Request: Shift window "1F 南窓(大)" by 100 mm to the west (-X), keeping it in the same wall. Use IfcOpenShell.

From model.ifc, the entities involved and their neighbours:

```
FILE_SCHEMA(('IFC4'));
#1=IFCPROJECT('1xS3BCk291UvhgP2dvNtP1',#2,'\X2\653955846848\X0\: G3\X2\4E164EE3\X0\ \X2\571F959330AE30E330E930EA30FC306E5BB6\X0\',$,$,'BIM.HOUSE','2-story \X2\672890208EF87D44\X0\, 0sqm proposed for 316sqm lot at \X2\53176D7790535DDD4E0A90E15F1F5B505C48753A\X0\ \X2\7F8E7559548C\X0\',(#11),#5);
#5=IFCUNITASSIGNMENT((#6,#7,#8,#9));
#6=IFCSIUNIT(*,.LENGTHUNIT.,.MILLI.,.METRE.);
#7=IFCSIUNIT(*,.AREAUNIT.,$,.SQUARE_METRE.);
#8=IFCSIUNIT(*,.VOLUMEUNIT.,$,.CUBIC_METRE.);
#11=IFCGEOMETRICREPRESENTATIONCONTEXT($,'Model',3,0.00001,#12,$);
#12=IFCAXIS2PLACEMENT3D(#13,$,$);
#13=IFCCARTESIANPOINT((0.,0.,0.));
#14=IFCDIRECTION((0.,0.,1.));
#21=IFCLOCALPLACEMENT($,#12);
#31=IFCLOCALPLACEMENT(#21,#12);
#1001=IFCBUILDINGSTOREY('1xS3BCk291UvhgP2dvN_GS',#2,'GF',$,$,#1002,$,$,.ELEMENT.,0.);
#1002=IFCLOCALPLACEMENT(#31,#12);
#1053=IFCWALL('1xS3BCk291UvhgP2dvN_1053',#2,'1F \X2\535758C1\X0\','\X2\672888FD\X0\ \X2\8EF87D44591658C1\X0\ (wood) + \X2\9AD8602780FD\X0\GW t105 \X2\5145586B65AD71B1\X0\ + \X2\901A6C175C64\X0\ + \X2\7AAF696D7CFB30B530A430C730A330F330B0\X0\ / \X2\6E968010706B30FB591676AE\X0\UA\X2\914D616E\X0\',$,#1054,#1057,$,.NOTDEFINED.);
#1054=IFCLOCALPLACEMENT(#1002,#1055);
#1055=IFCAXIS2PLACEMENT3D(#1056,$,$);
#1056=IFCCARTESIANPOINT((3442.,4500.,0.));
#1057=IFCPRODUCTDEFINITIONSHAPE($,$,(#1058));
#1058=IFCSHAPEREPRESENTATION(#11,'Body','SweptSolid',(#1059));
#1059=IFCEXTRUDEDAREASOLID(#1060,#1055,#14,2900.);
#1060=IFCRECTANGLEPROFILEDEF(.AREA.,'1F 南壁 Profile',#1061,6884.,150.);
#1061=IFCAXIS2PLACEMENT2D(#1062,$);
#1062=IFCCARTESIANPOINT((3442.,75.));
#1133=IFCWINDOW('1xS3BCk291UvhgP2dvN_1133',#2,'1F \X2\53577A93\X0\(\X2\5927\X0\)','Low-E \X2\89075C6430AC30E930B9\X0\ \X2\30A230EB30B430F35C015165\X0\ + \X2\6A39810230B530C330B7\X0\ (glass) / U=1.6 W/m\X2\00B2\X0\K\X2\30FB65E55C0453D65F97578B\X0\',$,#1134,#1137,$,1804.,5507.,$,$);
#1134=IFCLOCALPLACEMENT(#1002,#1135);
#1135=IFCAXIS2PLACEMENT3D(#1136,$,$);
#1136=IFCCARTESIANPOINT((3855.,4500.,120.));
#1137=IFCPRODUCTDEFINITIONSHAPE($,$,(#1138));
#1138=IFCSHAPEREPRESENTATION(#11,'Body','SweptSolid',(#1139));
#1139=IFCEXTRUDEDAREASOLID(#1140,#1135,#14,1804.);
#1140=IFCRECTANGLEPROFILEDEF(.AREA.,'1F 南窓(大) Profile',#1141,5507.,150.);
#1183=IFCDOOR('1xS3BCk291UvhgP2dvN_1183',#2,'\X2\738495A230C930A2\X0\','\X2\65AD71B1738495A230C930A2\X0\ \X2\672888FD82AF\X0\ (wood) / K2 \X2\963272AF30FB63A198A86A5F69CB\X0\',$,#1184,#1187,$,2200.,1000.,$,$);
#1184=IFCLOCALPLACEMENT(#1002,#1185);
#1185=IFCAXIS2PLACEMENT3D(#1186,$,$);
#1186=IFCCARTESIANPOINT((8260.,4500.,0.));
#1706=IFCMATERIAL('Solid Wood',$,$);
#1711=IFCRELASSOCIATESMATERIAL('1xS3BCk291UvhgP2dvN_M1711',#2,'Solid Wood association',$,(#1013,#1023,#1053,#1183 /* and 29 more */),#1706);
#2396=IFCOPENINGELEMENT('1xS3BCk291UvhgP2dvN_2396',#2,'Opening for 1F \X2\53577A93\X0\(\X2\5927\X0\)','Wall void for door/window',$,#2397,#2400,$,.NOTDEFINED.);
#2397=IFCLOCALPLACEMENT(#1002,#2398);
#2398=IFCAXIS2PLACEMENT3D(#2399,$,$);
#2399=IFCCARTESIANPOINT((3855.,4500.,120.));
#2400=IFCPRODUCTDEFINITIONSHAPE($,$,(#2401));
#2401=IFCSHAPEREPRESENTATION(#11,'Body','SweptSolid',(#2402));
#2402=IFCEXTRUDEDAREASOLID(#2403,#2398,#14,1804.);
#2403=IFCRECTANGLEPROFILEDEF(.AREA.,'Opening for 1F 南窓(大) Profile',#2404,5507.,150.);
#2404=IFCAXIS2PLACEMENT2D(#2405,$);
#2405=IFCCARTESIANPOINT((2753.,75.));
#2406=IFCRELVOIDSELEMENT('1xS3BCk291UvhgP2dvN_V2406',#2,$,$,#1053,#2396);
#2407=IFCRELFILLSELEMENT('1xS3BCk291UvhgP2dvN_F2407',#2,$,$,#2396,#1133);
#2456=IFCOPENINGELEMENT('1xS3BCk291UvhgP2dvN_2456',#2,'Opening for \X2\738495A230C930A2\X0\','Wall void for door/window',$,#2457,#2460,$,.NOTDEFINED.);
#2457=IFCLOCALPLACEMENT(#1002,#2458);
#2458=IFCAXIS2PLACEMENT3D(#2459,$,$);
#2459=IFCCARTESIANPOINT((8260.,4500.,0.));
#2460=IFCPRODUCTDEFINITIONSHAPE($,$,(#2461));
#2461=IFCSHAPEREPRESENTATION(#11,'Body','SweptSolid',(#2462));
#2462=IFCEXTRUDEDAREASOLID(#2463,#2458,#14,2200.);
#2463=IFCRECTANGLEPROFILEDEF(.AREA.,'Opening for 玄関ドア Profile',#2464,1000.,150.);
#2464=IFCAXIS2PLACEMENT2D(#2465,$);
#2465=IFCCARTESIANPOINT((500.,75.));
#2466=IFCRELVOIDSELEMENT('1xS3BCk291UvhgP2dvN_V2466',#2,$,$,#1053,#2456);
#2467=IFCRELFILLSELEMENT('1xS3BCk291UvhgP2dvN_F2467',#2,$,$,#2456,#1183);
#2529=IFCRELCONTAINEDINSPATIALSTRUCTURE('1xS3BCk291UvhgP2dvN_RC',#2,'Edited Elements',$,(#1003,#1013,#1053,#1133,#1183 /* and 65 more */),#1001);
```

```python
import ifcopenshell
import ifcopenshell.api.geometry
import ifcopenshell.util.placement
import ifcopenshell.util.unit

model = ifcopenshell.open("model.ifc")
unit_scale = ifcopenshell.util.unit.calculate_unit_scale(model)

window = model.by_guid("1xS3BCk291UvhgP2dvN_1133")
opening = window.FillsVoids[0].RelatingOpeningElement
wall = opening.VoidsElements[0].RelatingBuildingElement

wall_matrix = ifcopenshell.util.placement.get_local_placement(wall.ObjectPlacement)
shift = wall_matrix[:3, 0] * -0.1 / unit_scale
before = ifcopenshell.util.placement.get_local_placement(window.ObjectPlacement)[:3, 3].copy()

# The window is not placed relative to its opening, so move both.
for product in (opening, window):
    matrix = ifcopenshell.util.placement.get_local_placement(product.ObjectPlacement)
    matrix[:3, 3] += shift
    ifcopenshell.api.geometry.edit_object_placement(model, product=product, matrix=matrix, is_si=False)

after = ifcopenshell.util.placement.get_local_placement(window.ObjectPlacement)[:3, 3]
print("window moved by", (after - before).round(3) + 0.0)

model.write("model-out.ifc")
```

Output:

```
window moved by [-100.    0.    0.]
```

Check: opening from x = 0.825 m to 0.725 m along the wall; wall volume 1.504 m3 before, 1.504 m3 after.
